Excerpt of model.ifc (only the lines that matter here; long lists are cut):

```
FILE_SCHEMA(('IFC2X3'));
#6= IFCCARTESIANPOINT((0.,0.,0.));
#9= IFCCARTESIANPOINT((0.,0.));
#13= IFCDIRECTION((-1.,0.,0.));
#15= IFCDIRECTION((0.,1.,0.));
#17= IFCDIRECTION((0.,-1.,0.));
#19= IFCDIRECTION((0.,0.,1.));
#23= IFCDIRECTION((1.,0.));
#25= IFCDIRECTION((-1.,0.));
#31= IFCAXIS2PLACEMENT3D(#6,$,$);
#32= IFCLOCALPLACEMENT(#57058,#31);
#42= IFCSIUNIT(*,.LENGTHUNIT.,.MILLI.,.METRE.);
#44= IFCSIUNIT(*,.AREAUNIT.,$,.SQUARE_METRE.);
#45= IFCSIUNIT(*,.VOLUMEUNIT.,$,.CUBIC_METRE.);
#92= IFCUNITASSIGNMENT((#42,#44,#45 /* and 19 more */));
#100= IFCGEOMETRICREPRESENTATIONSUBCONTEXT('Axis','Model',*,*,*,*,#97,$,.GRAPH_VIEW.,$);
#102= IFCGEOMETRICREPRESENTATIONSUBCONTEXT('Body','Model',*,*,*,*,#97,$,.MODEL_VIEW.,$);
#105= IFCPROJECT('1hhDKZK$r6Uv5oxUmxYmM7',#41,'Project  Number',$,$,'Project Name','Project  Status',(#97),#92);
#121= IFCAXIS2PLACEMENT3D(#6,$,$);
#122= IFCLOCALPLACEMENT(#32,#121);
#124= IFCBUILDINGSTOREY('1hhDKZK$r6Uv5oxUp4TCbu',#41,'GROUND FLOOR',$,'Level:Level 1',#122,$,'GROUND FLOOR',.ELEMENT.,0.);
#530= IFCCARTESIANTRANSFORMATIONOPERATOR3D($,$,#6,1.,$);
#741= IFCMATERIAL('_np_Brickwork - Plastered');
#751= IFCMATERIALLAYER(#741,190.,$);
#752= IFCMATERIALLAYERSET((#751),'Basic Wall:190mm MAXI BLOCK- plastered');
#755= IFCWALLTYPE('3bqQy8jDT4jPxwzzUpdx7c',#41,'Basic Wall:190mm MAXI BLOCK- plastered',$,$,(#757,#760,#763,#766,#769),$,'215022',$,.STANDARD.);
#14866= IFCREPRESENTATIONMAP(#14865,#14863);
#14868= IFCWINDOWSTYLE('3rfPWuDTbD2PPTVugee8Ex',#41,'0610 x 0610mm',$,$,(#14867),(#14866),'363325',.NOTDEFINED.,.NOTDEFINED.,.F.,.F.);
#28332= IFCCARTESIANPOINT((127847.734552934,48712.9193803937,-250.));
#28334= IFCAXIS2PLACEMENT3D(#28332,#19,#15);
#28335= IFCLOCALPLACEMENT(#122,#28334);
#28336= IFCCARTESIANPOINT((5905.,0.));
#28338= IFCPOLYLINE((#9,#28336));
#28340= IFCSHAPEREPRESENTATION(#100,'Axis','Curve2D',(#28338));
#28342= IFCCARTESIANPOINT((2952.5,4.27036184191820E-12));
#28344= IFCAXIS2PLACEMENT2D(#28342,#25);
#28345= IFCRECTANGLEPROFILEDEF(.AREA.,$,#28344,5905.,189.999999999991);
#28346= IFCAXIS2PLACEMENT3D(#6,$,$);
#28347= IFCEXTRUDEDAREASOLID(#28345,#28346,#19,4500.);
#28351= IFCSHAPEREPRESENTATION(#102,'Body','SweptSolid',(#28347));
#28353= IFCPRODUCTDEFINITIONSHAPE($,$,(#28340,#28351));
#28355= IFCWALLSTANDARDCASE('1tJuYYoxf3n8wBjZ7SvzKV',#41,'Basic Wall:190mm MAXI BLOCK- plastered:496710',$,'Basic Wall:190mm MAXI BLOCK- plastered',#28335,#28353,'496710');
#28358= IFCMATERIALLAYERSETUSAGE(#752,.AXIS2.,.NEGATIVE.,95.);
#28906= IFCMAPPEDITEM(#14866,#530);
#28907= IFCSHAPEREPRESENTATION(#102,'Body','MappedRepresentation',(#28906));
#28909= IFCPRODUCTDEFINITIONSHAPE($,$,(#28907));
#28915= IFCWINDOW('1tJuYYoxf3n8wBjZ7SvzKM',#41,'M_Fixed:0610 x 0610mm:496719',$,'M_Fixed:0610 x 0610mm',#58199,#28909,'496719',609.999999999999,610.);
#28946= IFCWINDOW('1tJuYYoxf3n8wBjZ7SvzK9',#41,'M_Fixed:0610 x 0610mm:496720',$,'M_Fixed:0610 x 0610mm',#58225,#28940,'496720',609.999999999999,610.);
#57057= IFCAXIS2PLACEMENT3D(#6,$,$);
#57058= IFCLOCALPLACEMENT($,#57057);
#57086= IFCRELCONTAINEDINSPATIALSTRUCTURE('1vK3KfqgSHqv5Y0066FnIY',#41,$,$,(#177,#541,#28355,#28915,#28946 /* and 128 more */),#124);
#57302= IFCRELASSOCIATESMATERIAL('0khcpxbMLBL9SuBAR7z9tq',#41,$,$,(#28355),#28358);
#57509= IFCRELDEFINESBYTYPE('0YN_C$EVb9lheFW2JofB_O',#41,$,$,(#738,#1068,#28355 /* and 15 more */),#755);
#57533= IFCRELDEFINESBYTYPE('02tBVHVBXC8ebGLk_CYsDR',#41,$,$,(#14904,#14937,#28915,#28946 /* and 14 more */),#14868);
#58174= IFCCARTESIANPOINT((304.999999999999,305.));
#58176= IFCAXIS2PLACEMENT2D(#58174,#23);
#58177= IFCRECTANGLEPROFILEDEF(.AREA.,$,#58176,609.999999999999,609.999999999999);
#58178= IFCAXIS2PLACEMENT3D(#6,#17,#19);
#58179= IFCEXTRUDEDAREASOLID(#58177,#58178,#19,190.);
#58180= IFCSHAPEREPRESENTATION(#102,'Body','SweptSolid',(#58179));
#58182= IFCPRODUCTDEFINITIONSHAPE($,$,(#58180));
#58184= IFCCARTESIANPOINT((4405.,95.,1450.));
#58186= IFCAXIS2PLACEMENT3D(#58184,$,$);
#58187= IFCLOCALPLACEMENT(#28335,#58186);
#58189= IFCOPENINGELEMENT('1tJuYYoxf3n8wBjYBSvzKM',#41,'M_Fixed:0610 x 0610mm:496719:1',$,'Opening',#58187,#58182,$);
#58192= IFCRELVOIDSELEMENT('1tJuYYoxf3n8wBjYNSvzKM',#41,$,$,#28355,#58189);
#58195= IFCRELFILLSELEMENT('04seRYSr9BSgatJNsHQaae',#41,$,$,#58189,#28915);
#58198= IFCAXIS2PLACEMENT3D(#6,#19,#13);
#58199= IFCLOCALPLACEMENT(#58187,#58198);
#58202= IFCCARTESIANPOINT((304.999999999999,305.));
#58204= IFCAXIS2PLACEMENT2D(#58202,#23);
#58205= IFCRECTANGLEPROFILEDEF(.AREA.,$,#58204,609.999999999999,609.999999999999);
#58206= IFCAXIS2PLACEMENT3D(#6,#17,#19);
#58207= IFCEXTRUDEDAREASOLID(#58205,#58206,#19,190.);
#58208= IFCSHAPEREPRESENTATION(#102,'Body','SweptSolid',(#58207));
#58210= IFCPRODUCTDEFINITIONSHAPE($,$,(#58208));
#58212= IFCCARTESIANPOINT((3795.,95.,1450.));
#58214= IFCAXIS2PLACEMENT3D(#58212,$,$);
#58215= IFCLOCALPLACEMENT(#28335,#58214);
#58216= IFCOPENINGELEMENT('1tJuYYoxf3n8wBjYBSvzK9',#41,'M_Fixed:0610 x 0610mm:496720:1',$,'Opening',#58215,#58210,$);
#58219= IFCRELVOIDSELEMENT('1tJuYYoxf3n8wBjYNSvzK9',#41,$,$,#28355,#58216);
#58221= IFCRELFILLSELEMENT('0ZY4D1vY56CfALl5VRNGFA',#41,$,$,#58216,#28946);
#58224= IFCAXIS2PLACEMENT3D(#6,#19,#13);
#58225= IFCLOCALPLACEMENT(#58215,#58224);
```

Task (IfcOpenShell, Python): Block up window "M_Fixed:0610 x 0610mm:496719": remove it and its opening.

```python
import ifcopenshell
import ifcopenshell.api.feature
import ifcopenshell.api.root
import ifcopenshell.geom
import ifcopenshell.util.shape

model = ifcopenshell.open("model.ifc")
settings = ifcopenshell.geom.settings()


def volume(element):
    """Net volume in cubic metres, openings subtracted."""
    shape = ifcopenshell.geom.create_shape(settings, element)
    return ifcopenshell.util.shape.get_volume(shape.geometry)


window = model.by_guid("1tJuYYoxf3n8wBjZ7SvzKM")
opening = window.FillsVoids[0].RelatingOpeningElement
wall = opening.VoidsElements[0].RelatingBuildingElement
before = volume(wall)

ifcopenshell.api.root.remove_product(model, product=window)
ifcopenshell.api.feature.remove_feature(model, feature=opening)

after = volume(wall)

print(f"wall volume {before:.3f} -> {after:.3f} m3")

model.write("model_updated.ifc")
```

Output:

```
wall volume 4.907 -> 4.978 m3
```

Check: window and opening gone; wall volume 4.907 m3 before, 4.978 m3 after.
